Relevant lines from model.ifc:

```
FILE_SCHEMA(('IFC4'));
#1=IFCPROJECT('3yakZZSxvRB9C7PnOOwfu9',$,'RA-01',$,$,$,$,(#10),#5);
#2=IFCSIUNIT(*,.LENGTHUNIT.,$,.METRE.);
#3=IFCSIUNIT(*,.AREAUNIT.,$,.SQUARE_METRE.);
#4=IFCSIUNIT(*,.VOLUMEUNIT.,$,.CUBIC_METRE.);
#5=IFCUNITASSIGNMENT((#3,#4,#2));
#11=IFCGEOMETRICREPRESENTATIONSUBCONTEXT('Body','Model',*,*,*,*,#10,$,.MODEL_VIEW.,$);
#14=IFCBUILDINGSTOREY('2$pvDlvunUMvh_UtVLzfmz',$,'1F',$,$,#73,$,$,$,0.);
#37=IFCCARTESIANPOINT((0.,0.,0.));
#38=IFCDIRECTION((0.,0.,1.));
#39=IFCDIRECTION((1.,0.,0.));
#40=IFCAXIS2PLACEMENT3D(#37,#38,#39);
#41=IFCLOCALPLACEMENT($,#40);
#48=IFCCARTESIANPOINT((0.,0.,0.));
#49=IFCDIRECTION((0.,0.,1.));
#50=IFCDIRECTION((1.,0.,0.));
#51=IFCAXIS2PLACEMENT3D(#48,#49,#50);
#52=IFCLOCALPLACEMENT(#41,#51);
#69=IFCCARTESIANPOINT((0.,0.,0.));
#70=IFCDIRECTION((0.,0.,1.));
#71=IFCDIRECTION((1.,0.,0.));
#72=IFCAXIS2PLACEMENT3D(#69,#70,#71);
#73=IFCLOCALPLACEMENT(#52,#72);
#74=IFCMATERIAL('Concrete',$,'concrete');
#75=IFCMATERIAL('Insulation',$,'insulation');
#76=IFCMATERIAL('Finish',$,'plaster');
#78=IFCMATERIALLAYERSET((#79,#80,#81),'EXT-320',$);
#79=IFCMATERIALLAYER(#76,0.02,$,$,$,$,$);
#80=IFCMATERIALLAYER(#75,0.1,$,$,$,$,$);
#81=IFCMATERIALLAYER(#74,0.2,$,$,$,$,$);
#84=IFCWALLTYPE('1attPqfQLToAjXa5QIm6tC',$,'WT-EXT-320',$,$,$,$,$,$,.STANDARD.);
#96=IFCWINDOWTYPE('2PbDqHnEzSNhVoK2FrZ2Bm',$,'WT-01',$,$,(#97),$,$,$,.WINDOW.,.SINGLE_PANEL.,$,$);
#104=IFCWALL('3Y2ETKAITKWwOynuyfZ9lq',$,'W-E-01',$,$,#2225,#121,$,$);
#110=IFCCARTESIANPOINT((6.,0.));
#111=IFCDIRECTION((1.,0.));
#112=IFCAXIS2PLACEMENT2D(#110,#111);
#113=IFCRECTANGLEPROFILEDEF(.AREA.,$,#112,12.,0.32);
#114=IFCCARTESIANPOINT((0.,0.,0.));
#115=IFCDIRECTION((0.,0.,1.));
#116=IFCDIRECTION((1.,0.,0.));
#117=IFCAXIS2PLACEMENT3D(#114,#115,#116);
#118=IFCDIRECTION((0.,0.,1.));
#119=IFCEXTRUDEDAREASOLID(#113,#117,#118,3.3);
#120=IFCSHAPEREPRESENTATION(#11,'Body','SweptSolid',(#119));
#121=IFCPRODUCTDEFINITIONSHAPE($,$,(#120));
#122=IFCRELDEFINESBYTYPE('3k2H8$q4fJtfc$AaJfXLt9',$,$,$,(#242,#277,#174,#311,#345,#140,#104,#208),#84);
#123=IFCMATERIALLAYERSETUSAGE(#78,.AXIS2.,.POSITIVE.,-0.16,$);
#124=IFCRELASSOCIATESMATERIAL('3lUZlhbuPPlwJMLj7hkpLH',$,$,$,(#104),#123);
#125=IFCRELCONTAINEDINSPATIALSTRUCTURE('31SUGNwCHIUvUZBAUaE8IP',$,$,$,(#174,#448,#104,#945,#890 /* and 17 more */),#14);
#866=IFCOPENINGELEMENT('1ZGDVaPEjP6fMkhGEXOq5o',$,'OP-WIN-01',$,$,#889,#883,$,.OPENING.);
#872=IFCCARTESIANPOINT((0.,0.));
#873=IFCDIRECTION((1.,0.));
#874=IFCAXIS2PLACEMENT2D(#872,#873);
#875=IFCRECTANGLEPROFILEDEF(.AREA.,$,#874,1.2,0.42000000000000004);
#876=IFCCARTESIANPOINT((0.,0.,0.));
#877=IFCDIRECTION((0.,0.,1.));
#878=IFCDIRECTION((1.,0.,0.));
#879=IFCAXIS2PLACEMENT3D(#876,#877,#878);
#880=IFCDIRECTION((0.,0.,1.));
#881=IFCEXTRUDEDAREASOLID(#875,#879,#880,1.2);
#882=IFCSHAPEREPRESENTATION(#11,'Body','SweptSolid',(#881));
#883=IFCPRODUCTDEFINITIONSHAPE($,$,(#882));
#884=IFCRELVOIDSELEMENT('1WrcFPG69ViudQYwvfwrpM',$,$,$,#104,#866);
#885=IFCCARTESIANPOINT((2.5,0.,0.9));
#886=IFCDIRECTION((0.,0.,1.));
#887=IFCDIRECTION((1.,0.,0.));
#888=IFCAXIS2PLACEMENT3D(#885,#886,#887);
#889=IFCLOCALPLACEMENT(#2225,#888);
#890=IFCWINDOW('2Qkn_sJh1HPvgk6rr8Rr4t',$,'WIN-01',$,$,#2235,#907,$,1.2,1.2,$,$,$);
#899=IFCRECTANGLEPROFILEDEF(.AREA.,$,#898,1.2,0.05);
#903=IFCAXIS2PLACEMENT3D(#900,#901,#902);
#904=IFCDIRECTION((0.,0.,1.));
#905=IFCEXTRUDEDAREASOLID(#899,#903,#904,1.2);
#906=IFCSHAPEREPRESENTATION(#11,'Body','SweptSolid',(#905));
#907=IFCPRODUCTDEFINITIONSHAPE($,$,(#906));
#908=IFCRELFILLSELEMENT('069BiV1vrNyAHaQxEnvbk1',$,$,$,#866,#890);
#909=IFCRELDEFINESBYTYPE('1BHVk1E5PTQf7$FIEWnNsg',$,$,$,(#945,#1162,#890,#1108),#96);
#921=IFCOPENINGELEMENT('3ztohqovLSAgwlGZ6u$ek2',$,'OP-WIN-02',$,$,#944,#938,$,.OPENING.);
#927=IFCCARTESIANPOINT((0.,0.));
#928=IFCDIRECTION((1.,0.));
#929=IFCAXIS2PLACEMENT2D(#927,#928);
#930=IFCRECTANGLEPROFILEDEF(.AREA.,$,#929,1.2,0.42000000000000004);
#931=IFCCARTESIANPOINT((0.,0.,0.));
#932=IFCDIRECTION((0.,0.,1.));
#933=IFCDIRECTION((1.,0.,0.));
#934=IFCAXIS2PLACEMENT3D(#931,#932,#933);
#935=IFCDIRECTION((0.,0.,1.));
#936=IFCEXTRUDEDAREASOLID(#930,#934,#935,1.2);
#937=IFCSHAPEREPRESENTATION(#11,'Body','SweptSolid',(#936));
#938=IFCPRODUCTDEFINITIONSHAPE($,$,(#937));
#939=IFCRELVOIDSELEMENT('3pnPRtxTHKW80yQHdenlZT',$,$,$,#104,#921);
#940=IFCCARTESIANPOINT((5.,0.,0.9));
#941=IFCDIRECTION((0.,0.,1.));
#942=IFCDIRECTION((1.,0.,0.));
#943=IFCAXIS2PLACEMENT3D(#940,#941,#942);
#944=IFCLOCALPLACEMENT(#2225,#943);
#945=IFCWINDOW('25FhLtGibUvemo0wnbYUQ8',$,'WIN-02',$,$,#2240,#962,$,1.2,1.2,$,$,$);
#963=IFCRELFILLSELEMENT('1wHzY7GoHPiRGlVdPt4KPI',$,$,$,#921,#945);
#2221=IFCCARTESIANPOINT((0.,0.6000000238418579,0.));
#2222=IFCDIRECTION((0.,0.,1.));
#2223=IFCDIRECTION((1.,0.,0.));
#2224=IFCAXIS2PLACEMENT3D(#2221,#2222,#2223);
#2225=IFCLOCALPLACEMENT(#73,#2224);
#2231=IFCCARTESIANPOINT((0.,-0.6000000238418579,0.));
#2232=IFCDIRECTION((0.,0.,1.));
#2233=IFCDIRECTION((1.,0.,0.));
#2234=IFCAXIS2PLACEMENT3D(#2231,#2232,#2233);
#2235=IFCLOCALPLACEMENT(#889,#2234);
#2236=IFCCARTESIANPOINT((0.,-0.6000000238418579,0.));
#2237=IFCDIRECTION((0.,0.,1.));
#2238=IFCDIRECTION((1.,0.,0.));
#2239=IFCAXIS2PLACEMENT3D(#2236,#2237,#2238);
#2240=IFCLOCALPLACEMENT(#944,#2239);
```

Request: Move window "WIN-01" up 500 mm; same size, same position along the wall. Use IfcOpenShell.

```python
import numpy as np
import ifcopenshell
import ifcopenshell.api.geometry
import ifcopenshell.util.placement
import ifcopenshell.util.unit

model = ifcopenshell.open("model.ifc")
unit_scale = ifcopenshell.util.unit.calculate_unit_scale(model)

window = model.by_id(890)
opening = window.FillsVoids[0].RelatingOpeningElement
dz = 0.5 / unit_scale

shift = np.array([0.0, 0.0, dz])
# The window is placed relative to its opening, so it follows when the opening moves.
matrix = ifcopenshell.util.placement.get_local_placement(opening.ObjectPlacement)
matrix[:3, 3] += shift
ifcopenshell.api.geometry.edit_object_placement(
    model, product=opening, matrix=matrix, is_si=False, should_transform_children=True
)

print(f"moved by {dz * unit_scale:+.3f} m")

model.write("model_rev.ifc")
```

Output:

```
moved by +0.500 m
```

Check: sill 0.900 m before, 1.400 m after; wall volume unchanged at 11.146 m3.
